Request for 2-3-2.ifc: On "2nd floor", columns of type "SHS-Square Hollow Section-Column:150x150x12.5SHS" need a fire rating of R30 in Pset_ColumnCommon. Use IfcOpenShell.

First a look at what the model holds.

```python
import ifcopenshell
import ifcopenshell.util.element

model = ifcopenshell.open("2-3-2.ifc")
print(model.schema)
storey = next(s for s in model.by_type("IfcBuildingStorey") if s.Name == "2nd floor")
columns = [e for e in ifcopenshell.util.element.get_decomposition(storey) if e.is_a("IfcColumn")]
seen = {}
for e in columns:
    element_type = ifcopenshell.util.element.get_type(e)
    key = (element_type.Name if element_type != e and element_type else None, ifcopenshell.util.element.get_pset(e, "Pset_ColumnCommon", "FireRating"))
    seen[key] = seen.get(key, 0) + 1
for (name, value), count in sorted(seen.items(), key=str):
    print(count, "x", name, "|", value)
```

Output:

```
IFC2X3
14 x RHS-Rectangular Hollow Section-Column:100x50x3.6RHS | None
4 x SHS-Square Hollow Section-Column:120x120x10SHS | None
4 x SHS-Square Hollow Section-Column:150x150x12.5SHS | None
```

```python
import ifcopenshell
import ifcopenshell.api.pset
import ifcopenshell.util.element

model = ifcopenshell.open("2-3-2.ifc")

storey = next(s for s in model.by_type("IfcBuildingStorey") if s.Name == "2nd floor")
columns = [e for e in ifcopenshell.util.element.get_decomposition(storey) if e.is_a("IfcColumn")]

count = 0
for e in columns:
    element_type = ifcopenshell.util.element.get_type(e)
    if element_type in (None, e) or element_type.Name != "SHS-Square Hollow Section-Column:150x150x12.5SHS":
        continue
    # add_pset returns the element's existing set when there is one.
    pset = ifcopenshell.api.pset.add_pset(model, product=e, name="Pset_ColumnCommon")
    ifcopenshell.api.pset.edit_pset(model, pset=pset, properties={"FireRating": "R30"})
    count += 1

print(count, "columns updated")

model.write("2-3-2_rev.ifc")
```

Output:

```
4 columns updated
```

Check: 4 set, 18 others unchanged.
